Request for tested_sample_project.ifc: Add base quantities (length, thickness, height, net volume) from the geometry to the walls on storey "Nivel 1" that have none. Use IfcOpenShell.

First a look at what the model holds.

```python
import ifcopenshell
import ifcopenshell.util.element
import ifcopenshell.util.unit

model = ifcopenshell.open("tested_sample_project.ifc")
print(model.schema)
for unit_type in ("LENGTHUNIT", "AREAUNIT", "VOLUMEUNIT"):
    print(unit_type, ifcopenshell.util.unit.calculate_unit_scale(model, unit_type))
storey = next(s for s in model.by_type("IfcBuildingStorey") if s.Name == "Nivel 1")
walls = [e for e in ifcopenshell.util.element.get_decomposition(storey) if e.is_a("IfcWall")]
for e in sorted(walls, key=lambda e: e.id()):
    print(e.id(), e.is_a(), e.Name, list(ifcopenshell.util.element.get_psets(e, qtos_only=True)), sep=" | ")
```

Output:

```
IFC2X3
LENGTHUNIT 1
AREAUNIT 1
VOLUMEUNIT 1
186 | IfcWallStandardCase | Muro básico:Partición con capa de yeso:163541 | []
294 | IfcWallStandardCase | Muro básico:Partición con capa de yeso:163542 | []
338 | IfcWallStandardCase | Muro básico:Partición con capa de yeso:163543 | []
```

```python
import ifcopenshell
import ifcopenshell.api.pset
import ifcopenshell.geom
import ifcopenshell.util.element
import ifcopenshell.util.shape
import ifcopenshell.util.unit

model = ifcopenshell.open("tested_sample_project.ifc")
unit_scale = ifcopenshell.util.unit.calculate_unit_scale(model)
volume_scale = ifcopenshell.util.unit.calculate_unit_scale(model, "VOLUMEUNIT")
settings = ifcopenshell.geom.settings()

storey = next(s for s in model.by_type("IfcBuildingStorey") if s.Name == "Nivel 1")
walls = [e for e in ifcopenshell.util.element.get_decomposition(storey) if e.is_a("IfcWall")]

for e in sorted(walls, key=lambda e: e.id()):
    if ifcopenshell.util.element.get_psets(e, qtos_only=True, should_inherit=False):
        continue
    # Geometry comes back in metres, in the element's own axes.
    shape = ifcopenshell.geom.create_shape(settings, e)
    values = {
        "Length": ifcopenshell.util.shape.get_x(shape.geometry) / unit_scale,
        "Width": ifcopenshell.util.shape.get_y(shape.geometry) / unit_scale,
        "Height": ifcopenshell.util.shape.get_z(shape.geometry) / unit_scale,
        "NetVolume": ifcopenshell.util.shape.get_volume(shape.geometry) / volume_scale,
    }
    qto = ifcopenshell.api.pset.add_qto(model, product=e, name="BaseQuantities")
    ifcopenshell.api.pset.edit_qto(model, qto=qto, properties=values)
    print(e.id(), {k: round(v, 3) for k, v in values.items()})

model.write("tested_sample_project_rev.ifc")
```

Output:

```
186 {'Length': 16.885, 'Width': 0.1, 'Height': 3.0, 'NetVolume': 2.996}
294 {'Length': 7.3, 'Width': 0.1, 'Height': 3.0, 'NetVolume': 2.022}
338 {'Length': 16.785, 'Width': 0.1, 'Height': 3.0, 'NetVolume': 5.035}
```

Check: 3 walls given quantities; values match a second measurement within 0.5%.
